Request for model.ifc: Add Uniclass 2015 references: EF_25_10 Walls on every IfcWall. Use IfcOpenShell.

First a look at what the model holds.

```python
import ifcopenshell

model = ifcopenshell.open("model.ifc")
print(model.schema)
print("classifications:", [c.Name for c in model.by_type("IfcClassification")])
for ifc_class in ("IfcDoor", "IfcRoof", "IfcStair", "IfcWall", "IfcWindow"):
    print(ifc_class, len(model.by_type(ifc_class)))
```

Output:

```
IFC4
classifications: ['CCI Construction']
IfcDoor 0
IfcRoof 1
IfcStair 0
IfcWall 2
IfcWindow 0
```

```python
import ifcopenshell
import ifcopenshell.api.classification

model = ifcopenshell.open("model.ifc")

system = ifcopenshell.api.classification.add_classification(model, classification="Uniclass 2015")

codes = {
    "IfcWall": ("EF_25_10", "Walls"),
}
for ifc_class, (code, name) in codes.items():
    products = model.by_type(ifc_class)
    ifcopenshell.api.classification.add_reference(
        model, products=products, classification=system, identification=code, name=name
    )
    print(code, len(products))

model.write("model_edited.ifc")
```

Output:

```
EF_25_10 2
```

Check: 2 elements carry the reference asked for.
